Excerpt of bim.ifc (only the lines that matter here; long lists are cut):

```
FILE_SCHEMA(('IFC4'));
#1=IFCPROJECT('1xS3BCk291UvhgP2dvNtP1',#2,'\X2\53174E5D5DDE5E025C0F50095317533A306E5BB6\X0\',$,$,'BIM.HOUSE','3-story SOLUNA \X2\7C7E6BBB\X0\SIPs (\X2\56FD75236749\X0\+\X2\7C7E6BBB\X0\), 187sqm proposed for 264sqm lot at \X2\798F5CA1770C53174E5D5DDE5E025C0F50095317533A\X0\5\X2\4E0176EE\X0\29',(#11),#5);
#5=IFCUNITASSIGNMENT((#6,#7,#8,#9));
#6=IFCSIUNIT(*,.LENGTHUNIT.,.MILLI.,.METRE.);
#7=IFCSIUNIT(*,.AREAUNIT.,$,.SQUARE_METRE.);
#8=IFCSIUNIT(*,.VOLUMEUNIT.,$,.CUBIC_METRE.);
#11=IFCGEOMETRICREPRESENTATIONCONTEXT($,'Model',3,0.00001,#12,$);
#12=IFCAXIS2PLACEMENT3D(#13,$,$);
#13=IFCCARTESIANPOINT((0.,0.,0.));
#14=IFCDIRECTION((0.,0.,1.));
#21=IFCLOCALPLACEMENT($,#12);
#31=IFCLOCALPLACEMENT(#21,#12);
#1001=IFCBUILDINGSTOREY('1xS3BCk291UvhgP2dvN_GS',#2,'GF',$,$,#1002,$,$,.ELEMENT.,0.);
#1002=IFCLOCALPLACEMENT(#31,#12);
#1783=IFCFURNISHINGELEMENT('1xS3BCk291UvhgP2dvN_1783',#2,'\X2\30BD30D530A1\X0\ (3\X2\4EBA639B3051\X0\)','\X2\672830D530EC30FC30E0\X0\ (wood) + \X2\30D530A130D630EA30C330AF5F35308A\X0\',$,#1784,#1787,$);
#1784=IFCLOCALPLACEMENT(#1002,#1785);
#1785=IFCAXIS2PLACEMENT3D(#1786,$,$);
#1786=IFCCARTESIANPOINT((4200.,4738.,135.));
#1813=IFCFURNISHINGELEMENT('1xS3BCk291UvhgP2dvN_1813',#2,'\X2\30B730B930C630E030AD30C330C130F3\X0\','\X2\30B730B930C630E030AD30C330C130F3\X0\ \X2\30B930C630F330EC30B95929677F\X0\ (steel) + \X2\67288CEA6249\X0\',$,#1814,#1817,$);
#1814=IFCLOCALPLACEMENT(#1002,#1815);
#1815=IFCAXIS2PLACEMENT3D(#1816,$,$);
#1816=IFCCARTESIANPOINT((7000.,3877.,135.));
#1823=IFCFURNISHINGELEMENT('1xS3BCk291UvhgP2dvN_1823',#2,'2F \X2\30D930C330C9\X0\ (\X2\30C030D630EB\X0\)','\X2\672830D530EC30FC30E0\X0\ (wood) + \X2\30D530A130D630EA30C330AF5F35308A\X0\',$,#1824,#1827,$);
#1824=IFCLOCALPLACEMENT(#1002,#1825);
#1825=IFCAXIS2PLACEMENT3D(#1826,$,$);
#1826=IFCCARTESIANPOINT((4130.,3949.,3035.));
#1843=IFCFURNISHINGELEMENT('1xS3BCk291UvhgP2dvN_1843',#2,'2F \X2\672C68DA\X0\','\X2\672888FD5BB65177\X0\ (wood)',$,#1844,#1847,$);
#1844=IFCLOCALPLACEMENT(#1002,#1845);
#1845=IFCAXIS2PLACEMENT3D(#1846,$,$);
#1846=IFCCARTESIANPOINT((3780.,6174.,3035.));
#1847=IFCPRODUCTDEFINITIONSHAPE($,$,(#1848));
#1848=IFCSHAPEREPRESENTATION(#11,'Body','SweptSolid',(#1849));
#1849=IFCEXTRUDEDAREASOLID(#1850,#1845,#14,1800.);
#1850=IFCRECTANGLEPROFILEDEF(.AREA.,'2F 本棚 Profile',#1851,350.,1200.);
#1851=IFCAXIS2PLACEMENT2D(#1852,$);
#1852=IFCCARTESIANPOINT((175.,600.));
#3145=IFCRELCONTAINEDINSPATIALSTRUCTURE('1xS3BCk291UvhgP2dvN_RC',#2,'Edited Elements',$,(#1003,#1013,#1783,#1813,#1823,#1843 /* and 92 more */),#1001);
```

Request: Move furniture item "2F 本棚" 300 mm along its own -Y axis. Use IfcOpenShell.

```python
import ifcopenshell
import ifcopenshell.api.geometry
import ifcopenshell.util.placement

model = ifcopenshell.open("bim.ifc")

item = model.by_guid("1xS3BCk291UvhgP2dvN_1843")
matrix = ifcopenshell.util.placement.get_local_placement(item.ObjectPlacement)
matrix[:3, 3] -= matrix[:3, 1] * 300.0
ifcopenshell.api.geometry.edit_object_placement(model, product=item, matrix=matrix, is_si=False)

print(ifcopenshell.util.placement.get_local_placement(item.ObjectPlacement).round(3) + 0.0)

model.write("bim_v2.ifc")
```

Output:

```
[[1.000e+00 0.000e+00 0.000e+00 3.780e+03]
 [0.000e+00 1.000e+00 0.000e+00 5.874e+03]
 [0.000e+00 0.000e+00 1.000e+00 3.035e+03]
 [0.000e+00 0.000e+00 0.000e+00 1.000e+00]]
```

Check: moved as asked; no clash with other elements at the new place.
